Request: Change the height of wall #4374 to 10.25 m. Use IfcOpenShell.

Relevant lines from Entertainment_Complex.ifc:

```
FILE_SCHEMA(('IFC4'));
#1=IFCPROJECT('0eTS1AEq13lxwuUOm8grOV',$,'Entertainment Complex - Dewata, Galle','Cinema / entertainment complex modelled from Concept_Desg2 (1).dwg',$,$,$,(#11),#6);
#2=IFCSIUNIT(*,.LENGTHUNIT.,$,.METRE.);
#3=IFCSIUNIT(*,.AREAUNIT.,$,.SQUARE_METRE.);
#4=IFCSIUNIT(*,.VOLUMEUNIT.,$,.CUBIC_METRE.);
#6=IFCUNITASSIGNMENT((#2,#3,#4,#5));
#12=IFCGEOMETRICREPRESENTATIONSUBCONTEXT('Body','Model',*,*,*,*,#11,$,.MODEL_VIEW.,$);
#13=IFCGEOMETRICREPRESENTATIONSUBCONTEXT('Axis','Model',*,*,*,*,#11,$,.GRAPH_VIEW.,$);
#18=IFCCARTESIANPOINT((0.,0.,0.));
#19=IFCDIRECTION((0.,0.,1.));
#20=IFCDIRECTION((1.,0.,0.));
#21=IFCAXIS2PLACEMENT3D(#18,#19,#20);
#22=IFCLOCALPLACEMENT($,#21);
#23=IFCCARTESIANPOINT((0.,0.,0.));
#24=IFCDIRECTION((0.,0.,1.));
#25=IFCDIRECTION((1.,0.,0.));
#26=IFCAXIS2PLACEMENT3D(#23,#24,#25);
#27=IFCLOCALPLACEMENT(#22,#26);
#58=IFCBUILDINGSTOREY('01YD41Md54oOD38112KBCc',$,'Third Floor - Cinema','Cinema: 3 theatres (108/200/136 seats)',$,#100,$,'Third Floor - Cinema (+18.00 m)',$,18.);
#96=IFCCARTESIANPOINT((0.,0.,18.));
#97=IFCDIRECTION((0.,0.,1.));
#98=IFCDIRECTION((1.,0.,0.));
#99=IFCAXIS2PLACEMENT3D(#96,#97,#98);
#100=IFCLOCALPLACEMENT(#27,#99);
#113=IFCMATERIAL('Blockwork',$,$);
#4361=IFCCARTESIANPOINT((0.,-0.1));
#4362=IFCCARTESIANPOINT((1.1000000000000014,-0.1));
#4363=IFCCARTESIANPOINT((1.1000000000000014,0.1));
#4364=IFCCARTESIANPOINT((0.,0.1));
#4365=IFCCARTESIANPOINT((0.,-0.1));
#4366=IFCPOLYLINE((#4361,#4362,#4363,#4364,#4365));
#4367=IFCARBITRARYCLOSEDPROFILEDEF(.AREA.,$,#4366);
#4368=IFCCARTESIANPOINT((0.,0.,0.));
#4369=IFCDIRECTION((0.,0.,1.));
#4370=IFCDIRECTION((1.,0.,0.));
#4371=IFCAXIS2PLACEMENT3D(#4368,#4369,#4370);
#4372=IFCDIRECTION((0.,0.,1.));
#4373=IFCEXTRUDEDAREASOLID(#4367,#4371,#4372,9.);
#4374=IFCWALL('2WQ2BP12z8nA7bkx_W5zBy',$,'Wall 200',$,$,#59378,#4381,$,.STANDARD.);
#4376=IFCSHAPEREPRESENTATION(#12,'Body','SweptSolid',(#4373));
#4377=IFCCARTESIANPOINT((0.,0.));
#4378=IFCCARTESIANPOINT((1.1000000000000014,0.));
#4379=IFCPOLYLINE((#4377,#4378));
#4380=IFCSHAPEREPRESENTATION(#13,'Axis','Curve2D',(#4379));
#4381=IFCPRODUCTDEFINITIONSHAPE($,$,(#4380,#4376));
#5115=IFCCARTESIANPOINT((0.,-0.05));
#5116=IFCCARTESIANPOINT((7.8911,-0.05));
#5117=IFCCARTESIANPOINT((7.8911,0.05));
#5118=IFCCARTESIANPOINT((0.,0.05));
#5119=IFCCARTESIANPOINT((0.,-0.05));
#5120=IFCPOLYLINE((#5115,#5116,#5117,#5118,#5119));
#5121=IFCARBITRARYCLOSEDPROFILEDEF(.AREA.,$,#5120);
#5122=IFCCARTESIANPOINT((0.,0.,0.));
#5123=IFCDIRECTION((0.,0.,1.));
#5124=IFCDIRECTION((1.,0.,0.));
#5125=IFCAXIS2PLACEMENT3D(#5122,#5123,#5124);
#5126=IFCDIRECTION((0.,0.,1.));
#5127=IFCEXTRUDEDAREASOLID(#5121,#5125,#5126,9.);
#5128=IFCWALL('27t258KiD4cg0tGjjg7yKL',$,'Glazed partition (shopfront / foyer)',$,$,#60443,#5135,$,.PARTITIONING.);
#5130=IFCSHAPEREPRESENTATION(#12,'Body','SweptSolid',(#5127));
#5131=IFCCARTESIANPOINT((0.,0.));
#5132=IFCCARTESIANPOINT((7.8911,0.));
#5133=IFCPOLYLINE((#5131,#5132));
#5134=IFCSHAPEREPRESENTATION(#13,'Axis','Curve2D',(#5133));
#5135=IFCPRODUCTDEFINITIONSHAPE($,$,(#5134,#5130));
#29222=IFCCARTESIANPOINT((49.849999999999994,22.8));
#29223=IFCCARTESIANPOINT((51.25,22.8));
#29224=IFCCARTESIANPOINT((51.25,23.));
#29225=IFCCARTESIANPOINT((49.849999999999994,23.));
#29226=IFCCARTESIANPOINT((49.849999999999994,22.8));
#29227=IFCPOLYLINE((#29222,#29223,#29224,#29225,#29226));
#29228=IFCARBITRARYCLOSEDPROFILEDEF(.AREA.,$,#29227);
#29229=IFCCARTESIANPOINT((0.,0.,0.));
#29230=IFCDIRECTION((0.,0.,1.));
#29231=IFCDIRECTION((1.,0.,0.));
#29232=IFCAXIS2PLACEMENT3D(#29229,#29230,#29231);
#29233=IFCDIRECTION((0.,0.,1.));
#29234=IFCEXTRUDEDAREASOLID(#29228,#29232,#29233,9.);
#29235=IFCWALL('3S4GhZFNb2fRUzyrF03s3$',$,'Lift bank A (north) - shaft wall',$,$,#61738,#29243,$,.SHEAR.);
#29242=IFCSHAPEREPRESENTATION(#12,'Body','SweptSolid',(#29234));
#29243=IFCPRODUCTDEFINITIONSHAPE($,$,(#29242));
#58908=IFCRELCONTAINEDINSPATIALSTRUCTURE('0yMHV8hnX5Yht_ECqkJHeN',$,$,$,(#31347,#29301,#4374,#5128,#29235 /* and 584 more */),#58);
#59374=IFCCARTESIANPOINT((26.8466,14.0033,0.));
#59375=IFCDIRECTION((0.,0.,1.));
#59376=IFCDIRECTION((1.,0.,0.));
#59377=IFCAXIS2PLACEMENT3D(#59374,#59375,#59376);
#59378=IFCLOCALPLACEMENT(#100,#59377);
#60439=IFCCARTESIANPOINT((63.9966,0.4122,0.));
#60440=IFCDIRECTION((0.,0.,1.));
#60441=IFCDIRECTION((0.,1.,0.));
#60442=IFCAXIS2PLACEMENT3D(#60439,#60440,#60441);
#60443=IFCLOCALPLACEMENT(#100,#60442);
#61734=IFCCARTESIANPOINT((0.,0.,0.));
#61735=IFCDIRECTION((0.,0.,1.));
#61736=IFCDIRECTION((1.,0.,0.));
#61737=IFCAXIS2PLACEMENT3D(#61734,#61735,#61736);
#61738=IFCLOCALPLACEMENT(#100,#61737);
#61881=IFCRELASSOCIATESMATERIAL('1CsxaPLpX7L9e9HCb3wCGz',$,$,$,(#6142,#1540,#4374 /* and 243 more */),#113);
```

```python
import ifcopenshell
import ifcopenshell.geom
import ifcopenshell.util.representation
import ifcopenshell.util.shape
import ifcopenshell.util.unit

model = ifcopenshell.open("Entertainment_Complex.ifc")
unit_scale = ifcopenshell.util.unit.calculate_unit_scale(model)
settings = ifcopenshell.geom.settings()


def volume(element):
    """Net volume in cubic metres, openings subtracted."""
    shape = ifcopenshell.geom.create_shape(settings, element)
    return ifcopenshell.util.shape.get_volume(shape.geometry)


wall = model.by_guid("2WQ2BP12z8nA7bkx_W5zBy")
before = volume(wall)

body = ifcopenshell.util.representation.get_representation(wall, "Model", "Body")
solid = body.Items[0]
old_height = solid.Depth
solid.Depth = 10.25 / unit_scale
after = volume(wall)

print(f"height {old_height:g} -> {solid.Depth:g}, volume {before:.3f} -> {after:.3f} m3")

model.write("Entertainment_Complex_edited.ifc")
```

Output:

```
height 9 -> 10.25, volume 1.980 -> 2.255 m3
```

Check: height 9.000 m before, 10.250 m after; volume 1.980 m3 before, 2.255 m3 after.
